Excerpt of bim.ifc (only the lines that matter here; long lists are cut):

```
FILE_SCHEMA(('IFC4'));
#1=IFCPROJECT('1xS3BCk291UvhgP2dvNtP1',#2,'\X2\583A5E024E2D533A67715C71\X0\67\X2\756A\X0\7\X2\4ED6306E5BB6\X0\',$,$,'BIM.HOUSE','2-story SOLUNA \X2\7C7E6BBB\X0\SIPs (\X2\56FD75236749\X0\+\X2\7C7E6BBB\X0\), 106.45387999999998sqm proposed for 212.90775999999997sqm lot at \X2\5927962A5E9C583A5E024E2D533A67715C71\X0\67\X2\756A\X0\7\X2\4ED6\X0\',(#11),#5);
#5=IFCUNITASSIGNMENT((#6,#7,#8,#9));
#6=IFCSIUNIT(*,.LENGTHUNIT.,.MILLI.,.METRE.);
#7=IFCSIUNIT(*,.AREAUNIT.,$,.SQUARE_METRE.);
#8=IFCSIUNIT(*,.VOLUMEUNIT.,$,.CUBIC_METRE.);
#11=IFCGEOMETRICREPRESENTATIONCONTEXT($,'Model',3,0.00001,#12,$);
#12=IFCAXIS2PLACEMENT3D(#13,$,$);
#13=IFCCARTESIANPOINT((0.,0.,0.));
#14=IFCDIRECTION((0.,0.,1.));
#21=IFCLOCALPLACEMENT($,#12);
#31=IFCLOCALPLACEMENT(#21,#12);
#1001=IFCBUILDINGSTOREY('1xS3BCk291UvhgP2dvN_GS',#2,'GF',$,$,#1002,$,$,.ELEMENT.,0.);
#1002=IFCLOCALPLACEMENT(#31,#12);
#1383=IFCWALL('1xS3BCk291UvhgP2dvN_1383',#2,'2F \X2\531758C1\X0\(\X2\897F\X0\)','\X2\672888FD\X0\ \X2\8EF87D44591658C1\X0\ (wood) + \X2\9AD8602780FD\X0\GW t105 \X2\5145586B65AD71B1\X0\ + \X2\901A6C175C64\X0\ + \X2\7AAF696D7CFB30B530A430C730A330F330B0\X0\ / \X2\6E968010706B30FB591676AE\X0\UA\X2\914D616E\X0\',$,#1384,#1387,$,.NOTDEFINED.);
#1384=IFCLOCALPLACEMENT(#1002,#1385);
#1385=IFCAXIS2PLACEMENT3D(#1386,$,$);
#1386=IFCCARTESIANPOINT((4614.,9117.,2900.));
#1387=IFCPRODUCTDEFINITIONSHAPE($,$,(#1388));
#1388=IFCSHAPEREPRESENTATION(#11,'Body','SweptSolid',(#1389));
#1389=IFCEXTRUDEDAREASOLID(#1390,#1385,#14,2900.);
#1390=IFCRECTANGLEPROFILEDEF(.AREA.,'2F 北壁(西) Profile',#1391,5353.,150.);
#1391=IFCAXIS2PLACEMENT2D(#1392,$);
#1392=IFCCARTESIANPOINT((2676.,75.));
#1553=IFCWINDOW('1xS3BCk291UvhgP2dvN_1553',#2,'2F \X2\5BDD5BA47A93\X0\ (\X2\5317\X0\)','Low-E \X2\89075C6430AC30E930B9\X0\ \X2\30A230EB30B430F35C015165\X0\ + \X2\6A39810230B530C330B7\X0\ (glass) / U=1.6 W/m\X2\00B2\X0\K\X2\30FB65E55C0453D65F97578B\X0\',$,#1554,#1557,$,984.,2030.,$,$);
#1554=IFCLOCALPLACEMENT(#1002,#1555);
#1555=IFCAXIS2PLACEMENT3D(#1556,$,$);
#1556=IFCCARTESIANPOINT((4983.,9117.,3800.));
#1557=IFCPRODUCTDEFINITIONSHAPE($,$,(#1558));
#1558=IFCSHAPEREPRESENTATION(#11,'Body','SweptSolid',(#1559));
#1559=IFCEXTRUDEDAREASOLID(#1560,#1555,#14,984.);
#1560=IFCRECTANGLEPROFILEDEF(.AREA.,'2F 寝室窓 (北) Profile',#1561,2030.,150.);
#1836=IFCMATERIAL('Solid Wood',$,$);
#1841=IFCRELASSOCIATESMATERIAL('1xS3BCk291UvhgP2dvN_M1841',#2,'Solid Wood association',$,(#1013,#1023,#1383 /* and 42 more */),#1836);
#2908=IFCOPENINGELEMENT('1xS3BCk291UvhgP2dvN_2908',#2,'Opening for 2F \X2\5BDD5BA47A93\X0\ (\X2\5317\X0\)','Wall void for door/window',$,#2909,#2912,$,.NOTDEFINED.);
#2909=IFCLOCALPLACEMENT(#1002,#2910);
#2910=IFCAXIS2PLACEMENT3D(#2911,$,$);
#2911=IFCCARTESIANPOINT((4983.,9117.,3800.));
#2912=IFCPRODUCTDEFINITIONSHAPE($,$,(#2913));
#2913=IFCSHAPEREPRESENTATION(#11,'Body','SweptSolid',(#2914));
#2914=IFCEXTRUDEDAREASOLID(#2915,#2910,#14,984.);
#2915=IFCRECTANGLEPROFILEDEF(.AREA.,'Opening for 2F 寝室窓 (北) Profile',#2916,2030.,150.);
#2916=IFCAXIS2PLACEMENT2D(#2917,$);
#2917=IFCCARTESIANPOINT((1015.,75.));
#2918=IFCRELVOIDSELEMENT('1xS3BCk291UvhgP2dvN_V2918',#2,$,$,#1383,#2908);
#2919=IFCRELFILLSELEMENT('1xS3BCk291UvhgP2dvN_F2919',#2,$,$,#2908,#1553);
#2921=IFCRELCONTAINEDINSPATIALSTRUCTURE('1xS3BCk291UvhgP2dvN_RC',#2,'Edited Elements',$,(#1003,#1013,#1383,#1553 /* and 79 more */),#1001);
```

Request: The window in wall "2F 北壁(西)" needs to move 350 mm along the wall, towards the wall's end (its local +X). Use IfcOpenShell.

```python
import ifcopenshell
import ifcopenshell.api.geometry
import ifcopenshell.util.placement

model = ifcopenshell.open("bim.ifc")

window = model.by_id(1553)
opening = window.FillsVoids[0].RelatingOpeningElement
wall = opening.VoidsElements[0].RelatingBuildingElement

wall_matrix = ifcopenshell.util.placement.get_local_placement(wall.ObjectPlacement)
shift = wall_matrix[:3, 0] * 350.0
before = ifcopenshell.util.placement.get_local_placement(window.ObjectPlacement)[:3, 3].copy()

# The window is not placed relative to its opening, so move both.
for product in (opening, window):
    matrix = ifcopenshell.util.placement.get_local_placement(product.ObjectPlacement)
    matrix[:3, 3] += shift
    ifcopenshell.api.geometry.edit_object_placement(model, product=product, matrix=matrix, is_si=False)

after = ifcopenshell.util.placement.get_local_placement(window.ObjectPlacement)[:3, 3]
print("window moved by", (after - before).round(3) + 0.0)

model.write("bim_updated.ifc")
```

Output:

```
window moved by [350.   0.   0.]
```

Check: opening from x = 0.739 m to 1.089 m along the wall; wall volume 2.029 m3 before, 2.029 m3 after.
